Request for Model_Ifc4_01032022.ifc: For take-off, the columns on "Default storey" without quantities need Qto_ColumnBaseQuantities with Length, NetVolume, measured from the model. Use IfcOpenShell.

First a look at what the model holds.

```python
import ifcopenshell
import ifcopenshell.util.element
import ifcopenshell.util.unit

model = ifcopenshell.open("Model_Ifc4_01032022.ifc")
print(model.schema)
for unit_type in ("LENGTHUNIT", "AREAUNIT", "VOLUMEUNIT"):
    print(unit_type, ifcopenshell.util.unit.calculate_unit_scale(model, unit_type))
storey = next(s for s in model.by_type("IfcBuildingStorey") if s.Name == "Default storey")
columns = [e for e in ifcopenshell.util.element.get_decomposition(storey) if e.is_a("IfcColumn")]
for e in sorted(columns, key=lambda e: e.id()):
    print(e.id(), e.is_a(), e.Name, list(ifcopenshell.util.element.get_psets(e, qtos_only=True)), sep=" | ")
```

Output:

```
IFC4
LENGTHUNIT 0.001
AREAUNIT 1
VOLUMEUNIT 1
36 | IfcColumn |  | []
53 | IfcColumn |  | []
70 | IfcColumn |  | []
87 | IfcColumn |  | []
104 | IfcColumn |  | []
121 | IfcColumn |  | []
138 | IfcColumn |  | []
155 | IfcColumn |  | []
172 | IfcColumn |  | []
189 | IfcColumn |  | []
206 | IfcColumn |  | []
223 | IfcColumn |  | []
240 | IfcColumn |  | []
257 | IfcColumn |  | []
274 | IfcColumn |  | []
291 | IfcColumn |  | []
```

```python
import ifcopenshell
import ifcopenshell.api.pset
import ifcopenshell.geom
import ifcopenshell.util.element
import ifcopenshell.util.shape
import ifcopenshell.util.unit

model = ifcopenshell.open("Model_Ifc4_01032022.ifc")
unit_scale = ifcopenshell.util.unit.calculate_unit_scale(model)
volume_scale = ifcopenshell.util.unit.calculate_unit_scale(model, "VOLUMEUNIT")
settings = ifcopenshell.geom.settings()

storey = next(s for s in model.by_type("IfcBuildingStorey") if s.Name == "Default storey")
columns = [e for e in ifcopenshell.util.element.get_decomposition(storey) if e.is_a("IfcColumn")]

for e in sorted(columns, key=lambda e: e.id()):
    if ifcopenshell.util.element.get_psets(e, qtos_only=True, should_inherit=False):
        continue
    # Geometry comes back in metres, in the element's own axes.
    shape = ifcopenshell.geom.create_shape(settings, e)
    values = {
        "Length": ifcopenshell.util.shape.get_z(shape.geometry) / unit_scale,
        "NetVolume": ifcopenshell.util.shape.get_volume(shape.geometry) / volume_scale,
    }
    qto = ifcopenshell.api.pset.add_qto(model, product=e, name="Qto_ColumnBaseQuantities")
    ifcopenshell.api.pset.edit_qto(model, qto=qto, properties=values)
    print(e.id(), {k: round(v, 3) for k, v in values.items()})

model.write("Model_Ifc4_01032022_edited.ifc")
```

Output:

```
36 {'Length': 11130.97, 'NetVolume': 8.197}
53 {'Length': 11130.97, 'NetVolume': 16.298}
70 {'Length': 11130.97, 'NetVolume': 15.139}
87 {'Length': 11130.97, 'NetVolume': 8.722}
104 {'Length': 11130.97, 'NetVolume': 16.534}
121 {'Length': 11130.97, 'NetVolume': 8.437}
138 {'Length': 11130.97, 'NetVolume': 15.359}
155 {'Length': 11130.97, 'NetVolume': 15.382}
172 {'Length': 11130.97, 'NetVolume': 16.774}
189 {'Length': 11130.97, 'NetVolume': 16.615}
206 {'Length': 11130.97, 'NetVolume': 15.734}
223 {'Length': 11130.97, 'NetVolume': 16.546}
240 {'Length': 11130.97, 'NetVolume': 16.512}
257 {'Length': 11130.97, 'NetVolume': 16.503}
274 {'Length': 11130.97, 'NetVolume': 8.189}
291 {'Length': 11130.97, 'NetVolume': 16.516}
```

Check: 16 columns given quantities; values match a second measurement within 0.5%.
